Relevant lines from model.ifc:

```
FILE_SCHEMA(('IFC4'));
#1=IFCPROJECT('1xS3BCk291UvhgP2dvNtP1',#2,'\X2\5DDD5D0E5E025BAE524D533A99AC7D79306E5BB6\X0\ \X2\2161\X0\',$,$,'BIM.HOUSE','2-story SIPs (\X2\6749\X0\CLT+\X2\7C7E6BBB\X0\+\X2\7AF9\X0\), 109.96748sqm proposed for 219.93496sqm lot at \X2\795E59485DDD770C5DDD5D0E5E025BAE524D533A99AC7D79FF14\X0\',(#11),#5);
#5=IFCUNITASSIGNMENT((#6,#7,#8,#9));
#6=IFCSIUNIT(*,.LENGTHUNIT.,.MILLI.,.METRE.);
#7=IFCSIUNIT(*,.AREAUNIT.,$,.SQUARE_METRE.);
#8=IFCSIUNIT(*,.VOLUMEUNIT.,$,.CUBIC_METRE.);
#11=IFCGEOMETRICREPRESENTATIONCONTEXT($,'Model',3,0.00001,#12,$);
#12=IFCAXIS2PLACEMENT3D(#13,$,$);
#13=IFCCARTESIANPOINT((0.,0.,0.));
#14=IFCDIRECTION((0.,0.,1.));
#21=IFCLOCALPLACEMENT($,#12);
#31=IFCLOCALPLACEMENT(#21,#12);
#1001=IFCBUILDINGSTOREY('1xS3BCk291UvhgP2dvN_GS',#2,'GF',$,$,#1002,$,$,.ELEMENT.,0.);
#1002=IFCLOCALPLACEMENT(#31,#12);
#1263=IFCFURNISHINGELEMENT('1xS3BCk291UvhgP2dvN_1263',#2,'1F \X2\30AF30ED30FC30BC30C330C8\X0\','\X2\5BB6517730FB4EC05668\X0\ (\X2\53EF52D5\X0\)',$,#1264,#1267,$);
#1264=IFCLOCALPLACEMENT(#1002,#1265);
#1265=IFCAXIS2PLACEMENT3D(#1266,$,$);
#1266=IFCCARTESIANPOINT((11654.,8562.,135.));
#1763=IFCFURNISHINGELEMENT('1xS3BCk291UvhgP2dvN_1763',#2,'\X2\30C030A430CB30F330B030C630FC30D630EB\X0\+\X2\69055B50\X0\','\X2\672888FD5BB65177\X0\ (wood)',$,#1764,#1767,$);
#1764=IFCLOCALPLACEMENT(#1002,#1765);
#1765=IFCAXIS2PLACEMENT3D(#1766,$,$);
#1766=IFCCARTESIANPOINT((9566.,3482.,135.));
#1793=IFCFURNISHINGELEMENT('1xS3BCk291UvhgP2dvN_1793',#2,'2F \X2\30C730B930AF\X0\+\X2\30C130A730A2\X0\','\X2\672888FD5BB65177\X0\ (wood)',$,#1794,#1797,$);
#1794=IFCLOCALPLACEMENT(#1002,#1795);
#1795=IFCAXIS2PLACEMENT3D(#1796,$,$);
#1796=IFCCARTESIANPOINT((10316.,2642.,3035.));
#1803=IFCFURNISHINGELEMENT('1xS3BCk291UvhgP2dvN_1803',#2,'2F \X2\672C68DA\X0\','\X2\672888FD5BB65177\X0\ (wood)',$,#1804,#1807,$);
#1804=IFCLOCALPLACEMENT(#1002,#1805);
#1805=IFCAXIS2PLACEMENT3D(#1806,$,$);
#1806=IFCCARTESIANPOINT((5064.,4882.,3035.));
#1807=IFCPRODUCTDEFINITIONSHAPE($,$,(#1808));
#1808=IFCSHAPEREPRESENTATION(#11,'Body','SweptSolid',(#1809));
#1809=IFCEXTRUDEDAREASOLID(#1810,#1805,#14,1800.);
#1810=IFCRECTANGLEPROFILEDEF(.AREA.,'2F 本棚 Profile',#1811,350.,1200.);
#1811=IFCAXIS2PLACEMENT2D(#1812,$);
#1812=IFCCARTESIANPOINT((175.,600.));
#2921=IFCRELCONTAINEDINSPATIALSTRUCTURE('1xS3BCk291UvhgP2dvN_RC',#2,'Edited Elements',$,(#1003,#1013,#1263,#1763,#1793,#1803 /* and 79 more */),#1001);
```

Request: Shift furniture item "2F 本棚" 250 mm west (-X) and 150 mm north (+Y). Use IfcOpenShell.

```python
import ifcopenshell
import ifcopenshell.api.geometry
import ifcopenshell.util.placement
import ifcopenshell.util.unit

model = ifcopenshell.open("model.ifc")
unit_scale = ifcopenshell.util.unit.calculate_unit_scale(model)

item = model.by_guid("1xS3BCk291UvhgP2dvN_1803")
matrix = ifcopenshell.util.placement.get_local_placement(item.ObjectPlacement)
matrix[0, 3] -= 0.25 / unit_scale
matrix[1, 3] += 0.15 / unit_scale
ifcopenshell.api.geometry.edit_object_placement(model, product=item, matrix=matrix, is_si=False)

print(ifcopenshell.util.placement.get_local_placement(item.ObjectPlacement).round(3) + 0.0)

model.write("model-out.ifc")
```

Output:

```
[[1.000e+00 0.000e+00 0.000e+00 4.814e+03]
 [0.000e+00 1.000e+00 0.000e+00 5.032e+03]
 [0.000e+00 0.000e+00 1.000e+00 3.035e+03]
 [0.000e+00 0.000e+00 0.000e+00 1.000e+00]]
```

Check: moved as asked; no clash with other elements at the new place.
